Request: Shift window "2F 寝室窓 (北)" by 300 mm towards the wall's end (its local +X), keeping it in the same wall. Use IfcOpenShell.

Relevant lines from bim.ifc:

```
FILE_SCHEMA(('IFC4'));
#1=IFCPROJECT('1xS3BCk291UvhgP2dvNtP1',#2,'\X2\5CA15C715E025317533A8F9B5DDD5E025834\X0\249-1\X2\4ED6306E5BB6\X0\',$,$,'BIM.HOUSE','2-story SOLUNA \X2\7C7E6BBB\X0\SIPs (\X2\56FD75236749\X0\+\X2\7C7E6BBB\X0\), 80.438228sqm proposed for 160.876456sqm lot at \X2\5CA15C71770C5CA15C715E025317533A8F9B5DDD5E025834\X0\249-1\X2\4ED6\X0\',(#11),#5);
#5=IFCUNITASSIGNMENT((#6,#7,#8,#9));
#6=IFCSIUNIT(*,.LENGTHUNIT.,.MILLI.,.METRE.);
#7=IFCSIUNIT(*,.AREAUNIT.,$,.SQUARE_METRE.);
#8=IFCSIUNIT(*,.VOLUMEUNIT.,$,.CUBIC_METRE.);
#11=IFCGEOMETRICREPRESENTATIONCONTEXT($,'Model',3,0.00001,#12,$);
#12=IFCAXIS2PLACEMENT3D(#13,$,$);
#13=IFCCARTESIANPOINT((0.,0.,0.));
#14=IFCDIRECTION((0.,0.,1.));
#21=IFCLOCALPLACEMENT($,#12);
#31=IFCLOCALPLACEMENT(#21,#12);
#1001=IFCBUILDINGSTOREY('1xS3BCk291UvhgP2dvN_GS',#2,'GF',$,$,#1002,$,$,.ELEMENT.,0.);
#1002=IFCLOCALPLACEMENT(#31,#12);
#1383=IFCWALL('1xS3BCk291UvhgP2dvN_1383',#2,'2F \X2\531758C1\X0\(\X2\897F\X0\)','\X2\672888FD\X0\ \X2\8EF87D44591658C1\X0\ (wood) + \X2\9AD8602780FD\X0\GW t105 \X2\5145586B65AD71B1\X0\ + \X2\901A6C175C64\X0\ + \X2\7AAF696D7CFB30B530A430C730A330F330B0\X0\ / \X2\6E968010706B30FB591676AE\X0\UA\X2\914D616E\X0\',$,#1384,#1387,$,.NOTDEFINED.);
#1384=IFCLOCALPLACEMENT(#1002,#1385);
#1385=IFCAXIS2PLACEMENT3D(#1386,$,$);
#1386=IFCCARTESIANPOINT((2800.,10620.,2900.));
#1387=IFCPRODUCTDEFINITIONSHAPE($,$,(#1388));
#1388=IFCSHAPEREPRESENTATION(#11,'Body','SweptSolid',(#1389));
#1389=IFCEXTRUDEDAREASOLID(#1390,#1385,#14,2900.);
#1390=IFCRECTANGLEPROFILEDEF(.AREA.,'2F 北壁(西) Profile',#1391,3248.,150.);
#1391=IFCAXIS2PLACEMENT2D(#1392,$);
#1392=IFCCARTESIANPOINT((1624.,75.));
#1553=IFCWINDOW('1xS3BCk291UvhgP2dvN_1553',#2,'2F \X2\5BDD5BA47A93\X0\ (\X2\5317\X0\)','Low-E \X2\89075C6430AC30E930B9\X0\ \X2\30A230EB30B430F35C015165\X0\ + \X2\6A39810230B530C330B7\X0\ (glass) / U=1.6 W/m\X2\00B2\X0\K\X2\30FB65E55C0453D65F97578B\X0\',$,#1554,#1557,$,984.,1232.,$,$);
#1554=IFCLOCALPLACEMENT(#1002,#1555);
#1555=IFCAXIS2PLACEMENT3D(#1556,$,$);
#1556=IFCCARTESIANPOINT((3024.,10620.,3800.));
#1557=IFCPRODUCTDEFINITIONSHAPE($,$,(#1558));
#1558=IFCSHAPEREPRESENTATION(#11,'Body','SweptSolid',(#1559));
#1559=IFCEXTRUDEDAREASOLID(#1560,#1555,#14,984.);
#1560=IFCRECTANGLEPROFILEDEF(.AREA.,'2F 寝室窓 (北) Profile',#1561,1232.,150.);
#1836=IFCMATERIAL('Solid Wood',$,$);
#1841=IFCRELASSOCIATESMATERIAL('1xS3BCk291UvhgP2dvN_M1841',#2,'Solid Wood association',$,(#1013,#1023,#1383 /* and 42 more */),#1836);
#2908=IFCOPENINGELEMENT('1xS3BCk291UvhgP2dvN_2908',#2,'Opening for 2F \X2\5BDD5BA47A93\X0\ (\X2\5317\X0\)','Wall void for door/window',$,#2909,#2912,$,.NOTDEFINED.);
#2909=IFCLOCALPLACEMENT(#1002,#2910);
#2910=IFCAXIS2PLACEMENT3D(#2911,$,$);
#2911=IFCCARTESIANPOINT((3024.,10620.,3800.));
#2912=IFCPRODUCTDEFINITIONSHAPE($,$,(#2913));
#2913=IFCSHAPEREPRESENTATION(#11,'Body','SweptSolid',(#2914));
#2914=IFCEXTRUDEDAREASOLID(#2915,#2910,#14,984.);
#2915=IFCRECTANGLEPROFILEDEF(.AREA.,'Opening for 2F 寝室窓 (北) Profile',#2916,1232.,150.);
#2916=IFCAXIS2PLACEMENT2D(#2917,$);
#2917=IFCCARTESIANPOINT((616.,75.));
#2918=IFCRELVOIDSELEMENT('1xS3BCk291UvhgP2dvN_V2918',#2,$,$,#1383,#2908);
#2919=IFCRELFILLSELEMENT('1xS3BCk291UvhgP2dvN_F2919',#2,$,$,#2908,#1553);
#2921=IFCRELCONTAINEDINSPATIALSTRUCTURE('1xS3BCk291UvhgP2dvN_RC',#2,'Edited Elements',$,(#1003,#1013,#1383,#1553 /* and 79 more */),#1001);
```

```python
import ifcopenshell
import ifcopenshell.api.geometry
import ifcopenshell.util.placement
import ifcopenshell.util.unit

model = ifcopenshell.open("bim.ifc")
unit_scale = ifcopenshell.util.unit.calculate_unit_scale(model)

window = model.by_guid("1xS3BCk291UvhgP2dvN_1553")
opening = window.FillsVoids[0].RelatingOpeningElement
wall = opening.VoidsElements[0].RelatingBuildingElement

wall_matrix = ifcopenshell.util.placement.get_local_placement(wall.ObjectPlacement)
shift = wall_matrix[:3, 0] * 0.3 / unit_scale
before = ifcopenshell.util.placement.get_local_placement(window.ObjectPlacement)[:3, 3].copy()

# The window is not placed relative to its opening, so move both.
for product in (opening, window):
    matrix = ifcopenshell.util.placement.get_local_placement(product.ObjectPlacement)
    matrix[:3, 3] += shift
    ifcopenshell.api.geometry.edit_object_placement(model, product=product, matrix=matrix, is_si=False)

after = ifcopenshell.util.placement.get_local_placement(window.ObjectPlacement)[:3, 3]
print("window moved by", (after - before).round(3) + 0.0)

model.write("bim_updated.ifc")
```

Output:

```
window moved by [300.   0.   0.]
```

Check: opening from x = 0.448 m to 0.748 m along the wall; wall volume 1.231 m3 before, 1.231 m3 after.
